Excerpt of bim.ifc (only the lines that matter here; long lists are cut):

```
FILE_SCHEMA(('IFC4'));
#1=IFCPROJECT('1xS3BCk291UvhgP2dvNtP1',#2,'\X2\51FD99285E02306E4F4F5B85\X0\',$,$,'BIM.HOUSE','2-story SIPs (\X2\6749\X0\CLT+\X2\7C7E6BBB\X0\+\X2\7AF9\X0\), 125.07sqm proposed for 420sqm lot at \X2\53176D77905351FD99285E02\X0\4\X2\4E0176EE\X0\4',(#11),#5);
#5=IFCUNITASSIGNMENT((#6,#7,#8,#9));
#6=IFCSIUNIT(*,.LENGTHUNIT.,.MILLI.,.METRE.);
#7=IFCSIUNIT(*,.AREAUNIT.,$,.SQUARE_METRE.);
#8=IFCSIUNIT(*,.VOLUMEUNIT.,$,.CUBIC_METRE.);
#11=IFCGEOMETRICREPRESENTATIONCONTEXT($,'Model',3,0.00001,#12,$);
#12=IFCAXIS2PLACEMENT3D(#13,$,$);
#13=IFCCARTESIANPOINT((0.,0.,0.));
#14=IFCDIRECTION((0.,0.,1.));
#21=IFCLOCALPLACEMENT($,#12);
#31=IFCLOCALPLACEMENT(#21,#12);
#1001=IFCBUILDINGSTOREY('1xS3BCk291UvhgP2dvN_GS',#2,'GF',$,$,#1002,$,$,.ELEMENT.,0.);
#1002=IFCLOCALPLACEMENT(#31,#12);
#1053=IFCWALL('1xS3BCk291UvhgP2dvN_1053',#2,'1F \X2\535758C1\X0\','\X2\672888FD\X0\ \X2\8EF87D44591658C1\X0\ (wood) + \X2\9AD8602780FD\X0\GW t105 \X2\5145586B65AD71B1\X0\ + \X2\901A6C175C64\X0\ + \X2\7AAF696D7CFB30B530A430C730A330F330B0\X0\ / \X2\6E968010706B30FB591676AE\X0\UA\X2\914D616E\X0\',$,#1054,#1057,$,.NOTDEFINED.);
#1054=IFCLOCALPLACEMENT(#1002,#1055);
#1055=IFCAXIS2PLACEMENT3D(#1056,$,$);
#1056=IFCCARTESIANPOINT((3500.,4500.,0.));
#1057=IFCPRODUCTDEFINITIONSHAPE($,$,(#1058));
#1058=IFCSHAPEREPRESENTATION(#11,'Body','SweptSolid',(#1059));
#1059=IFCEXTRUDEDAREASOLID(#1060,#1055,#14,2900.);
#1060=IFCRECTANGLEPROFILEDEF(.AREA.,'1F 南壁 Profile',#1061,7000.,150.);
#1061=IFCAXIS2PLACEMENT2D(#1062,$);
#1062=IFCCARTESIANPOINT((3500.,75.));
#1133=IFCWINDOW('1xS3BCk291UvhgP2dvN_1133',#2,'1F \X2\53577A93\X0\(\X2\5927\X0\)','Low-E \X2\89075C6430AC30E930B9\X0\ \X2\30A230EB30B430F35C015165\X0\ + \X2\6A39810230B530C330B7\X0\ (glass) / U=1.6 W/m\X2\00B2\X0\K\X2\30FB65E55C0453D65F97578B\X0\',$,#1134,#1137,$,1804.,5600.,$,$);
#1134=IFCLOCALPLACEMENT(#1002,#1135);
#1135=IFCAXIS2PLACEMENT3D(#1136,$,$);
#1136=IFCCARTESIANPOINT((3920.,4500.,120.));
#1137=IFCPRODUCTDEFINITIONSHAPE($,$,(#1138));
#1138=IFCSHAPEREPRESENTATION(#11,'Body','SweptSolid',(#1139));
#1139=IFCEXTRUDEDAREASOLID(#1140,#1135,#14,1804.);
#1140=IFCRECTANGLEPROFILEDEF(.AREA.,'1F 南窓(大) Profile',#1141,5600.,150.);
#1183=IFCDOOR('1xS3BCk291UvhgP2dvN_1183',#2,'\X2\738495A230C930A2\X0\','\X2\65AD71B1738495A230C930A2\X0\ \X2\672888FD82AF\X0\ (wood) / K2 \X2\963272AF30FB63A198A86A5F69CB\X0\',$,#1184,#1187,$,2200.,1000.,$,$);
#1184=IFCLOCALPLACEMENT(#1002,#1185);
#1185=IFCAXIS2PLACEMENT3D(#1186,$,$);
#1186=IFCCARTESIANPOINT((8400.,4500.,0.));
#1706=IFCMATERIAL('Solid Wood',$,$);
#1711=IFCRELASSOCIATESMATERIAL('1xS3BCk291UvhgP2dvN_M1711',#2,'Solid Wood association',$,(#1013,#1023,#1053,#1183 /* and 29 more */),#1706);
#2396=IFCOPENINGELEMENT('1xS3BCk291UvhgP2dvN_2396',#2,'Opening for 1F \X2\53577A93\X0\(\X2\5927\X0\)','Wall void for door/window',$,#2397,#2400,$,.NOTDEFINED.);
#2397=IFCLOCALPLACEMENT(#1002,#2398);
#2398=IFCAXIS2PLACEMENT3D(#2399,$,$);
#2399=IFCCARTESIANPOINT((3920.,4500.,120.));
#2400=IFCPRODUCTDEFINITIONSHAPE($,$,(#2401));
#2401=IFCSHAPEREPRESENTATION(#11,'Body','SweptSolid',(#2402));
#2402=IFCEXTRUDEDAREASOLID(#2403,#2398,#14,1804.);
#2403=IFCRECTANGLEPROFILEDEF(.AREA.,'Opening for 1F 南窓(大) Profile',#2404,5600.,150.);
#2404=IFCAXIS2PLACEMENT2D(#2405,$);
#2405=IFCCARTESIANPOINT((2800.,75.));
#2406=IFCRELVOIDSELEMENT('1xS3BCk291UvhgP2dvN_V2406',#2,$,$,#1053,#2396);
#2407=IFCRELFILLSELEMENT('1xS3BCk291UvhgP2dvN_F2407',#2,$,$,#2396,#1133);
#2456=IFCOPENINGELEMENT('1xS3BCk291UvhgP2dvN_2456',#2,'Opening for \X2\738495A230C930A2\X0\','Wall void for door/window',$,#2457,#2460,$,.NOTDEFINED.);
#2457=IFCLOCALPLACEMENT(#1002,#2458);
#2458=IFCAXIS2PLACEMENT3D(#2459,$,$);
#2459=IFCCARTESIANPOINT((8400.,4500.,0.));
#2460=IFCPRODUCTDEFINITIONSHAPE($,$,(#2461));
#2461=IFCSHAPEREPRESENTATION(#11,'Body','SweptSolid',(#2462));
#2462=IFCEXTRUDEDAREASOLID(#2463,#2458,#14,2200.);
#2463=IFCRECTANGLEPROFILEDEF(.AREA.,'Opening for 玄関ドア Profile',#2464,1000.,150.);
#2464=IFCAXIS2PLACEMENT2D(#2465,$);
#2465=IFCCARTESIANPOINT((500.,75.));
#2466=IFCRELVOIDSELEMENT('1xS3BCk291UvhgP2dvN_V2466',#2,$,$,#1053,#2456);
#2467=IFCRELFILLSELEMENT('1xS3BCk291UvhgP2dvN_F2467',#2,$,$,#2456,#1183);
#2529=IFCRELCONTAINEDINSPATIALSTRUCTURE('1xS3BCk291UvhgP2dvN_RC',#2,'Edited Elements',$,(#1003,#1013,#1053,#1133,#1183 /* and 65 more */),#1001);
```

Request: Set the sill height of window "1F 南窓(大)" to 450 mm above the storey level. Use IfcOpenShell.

```python
import numpy as np
import ifcopenshell
import ifcopenshell.api.geometry
import ifcopenshell.geom
import ifcopenshell.util.element
import ifcopenshell.util.placement
import ifcopenshell.util.shape
import ifcopenshell.util.unit

model = ifcopenshell.open("bim.ifc")
unit_scale = ifcopenshell.util.unit.calculate_unit_scale(model)

window = model.by_id(1133)
opening = window.FillsVoids[0].RelatingOpeningElement
storey = ifcopenshell.util.element.get_container(window, ifc_class="IfcBuildingStorey")
level = ifcopenshell.util.placement.get_local_placement(storey.ObjectPlacement)[2, 3]

# The opening's origin need not be at the sill, so measure its lowest point.
shape = ifcopenshell.geom.create_shape(ifcopenshell.geom.settings(), opening)
bottom = ifcopenshell.util.shape.get_shape_bottom_elevation(shape, shape.geometry) / unit_scale
dz = level + 450.0 - bottom

shift = np.array([0.0, 0.0, dz])
# The window is not placed relative to its opening, so move both.
for product in (opening, window):
    matrix = ifcopenshell.util.placement.get_local_placement(product.ObjectPlacement)
    matrix[:3, 3] += shift
    ifcopenshell.api.geometry.edit_object_placement(model, product=product, matrix=matrix, is_si=False)

print(f"moved by {dz * unit_scale:+.3f} m")

model.write("bim_edited.ifc")
```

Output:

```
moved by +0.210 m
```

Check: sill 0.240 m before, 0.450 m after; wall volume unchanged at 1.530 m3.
